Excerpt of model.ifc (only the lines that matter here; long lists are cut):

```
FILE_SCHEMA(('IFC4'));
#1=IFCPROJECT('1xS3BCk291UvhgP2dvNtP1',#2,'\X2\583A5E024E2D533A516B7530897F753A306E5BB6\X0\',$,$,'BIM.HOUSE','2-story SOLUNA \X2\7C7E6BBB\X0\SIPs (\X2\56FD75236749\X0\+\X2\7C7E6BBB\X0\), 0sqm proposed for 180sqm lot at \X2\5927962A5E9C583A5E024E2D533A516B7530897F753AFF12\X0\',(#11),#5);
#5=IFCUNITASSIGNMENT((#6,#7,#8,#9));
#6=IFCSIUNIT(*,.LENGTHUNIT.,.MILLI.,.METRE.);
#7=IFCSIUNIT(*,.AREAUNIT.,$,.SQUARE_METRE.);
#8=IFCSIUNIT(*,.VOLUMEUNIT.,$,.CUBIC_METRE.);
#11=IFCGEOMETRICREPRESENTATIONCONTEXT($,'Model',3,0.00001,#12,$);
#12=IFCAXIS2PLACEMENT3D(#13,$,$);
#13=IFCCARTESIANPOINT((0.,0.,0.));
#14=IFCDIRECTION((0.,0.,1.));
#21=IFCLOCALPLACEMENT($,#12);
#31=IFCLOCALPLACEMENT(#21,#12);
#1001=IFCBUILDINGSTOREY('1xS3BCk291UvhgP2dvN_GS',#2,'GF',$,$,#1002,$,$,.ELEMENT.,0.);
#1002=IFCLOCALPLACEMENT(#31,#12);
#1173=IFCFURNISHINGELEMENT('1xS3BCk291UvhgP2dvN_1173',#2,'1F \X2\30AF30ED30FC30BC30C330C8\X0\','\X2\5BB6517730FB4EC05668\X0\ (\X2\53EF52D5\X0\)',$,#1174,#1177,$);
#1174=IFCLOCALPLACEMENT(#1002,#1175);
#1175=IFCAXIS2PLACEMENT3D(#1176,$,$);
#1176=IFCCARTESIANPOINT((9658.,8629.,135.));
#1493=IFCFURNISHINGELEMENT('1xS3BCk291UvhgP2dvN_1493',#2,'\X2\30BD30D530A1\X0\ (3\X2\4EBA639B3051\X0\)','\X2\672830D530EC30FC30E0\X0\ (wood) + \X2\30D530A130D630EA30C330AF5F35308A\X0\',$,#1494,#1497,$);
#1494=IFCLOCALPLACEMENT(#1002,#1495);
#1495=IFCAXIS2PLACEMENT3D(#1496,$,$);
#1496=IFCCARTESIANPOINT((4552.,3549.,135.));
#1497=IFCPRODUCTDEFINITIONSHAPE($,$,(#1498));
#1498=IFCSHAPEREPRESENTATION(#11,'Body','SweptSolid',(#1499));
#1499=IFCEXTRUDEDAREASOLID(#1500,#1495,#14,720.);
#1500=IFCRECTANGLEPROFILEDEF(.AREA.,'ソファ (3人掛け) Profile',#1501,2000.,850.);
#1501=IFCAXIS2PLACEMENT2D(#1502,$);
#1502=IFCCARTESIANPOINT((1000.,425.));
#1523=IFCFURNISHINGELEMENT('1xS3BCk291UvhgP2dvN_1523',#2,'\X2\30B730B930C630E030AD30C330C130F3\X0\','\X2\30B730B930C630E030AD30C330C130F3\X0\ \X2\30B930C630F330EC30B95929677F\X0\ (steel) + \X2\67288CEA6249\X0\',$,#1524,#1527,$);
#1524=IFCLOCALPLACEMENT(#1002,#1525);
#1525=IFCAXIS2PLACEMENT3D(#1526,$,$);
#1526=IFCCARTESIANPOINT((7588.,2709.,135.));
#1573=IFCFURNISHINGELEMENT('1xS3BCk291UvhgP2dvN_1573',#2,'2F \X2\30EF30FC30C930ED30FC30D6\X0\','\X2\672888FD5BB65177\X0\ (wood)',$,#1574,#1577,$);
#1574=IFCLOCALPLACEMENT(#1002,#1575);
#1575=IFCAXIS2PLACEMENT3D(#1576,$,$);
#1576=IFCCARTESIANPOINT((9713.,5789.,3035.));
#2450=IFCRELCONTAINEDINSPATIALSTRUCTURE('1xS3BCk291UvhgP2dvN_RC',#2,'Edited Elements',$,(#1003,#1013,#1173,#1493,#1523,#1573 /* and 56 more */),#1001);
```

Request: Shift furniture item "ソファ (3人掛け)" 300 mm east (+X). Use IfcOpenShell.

```python
import ifcopenshell
import ifcopenshell.api.geometry
import ifcopenshell.util.placement
import ifcopenshell.util.unit

model = ifcopenshell.open("model.ifc")
unit_scale = ifcopenshell.util.unit.calculate_unit_scale(model)

item = model.by_guid("1xS3BCk291UvhgP2dvN_1493")
matrix = ifcopenshell.util.placement.get_local_placement(item.ObjectPlacement)
matrix[0, 3] += 0.3 / unit_scale
ifcopenshell.api.geometry.edit_object_placement(model, product=item, matrix=matrix, is_si=False)

print(ifcopenshell.util.placement.get_local_placement(item.ObjectPlacement).round(3) + 0.0)

model.write("model_updated.ifc")
```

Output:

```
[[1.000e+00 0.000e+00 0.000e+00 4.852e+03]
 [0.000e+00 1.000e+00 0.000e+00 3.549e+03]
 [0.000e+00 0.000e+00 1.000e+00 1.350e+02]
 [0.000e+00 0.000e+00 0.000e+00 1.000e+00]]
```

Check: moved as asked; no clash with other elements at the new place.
